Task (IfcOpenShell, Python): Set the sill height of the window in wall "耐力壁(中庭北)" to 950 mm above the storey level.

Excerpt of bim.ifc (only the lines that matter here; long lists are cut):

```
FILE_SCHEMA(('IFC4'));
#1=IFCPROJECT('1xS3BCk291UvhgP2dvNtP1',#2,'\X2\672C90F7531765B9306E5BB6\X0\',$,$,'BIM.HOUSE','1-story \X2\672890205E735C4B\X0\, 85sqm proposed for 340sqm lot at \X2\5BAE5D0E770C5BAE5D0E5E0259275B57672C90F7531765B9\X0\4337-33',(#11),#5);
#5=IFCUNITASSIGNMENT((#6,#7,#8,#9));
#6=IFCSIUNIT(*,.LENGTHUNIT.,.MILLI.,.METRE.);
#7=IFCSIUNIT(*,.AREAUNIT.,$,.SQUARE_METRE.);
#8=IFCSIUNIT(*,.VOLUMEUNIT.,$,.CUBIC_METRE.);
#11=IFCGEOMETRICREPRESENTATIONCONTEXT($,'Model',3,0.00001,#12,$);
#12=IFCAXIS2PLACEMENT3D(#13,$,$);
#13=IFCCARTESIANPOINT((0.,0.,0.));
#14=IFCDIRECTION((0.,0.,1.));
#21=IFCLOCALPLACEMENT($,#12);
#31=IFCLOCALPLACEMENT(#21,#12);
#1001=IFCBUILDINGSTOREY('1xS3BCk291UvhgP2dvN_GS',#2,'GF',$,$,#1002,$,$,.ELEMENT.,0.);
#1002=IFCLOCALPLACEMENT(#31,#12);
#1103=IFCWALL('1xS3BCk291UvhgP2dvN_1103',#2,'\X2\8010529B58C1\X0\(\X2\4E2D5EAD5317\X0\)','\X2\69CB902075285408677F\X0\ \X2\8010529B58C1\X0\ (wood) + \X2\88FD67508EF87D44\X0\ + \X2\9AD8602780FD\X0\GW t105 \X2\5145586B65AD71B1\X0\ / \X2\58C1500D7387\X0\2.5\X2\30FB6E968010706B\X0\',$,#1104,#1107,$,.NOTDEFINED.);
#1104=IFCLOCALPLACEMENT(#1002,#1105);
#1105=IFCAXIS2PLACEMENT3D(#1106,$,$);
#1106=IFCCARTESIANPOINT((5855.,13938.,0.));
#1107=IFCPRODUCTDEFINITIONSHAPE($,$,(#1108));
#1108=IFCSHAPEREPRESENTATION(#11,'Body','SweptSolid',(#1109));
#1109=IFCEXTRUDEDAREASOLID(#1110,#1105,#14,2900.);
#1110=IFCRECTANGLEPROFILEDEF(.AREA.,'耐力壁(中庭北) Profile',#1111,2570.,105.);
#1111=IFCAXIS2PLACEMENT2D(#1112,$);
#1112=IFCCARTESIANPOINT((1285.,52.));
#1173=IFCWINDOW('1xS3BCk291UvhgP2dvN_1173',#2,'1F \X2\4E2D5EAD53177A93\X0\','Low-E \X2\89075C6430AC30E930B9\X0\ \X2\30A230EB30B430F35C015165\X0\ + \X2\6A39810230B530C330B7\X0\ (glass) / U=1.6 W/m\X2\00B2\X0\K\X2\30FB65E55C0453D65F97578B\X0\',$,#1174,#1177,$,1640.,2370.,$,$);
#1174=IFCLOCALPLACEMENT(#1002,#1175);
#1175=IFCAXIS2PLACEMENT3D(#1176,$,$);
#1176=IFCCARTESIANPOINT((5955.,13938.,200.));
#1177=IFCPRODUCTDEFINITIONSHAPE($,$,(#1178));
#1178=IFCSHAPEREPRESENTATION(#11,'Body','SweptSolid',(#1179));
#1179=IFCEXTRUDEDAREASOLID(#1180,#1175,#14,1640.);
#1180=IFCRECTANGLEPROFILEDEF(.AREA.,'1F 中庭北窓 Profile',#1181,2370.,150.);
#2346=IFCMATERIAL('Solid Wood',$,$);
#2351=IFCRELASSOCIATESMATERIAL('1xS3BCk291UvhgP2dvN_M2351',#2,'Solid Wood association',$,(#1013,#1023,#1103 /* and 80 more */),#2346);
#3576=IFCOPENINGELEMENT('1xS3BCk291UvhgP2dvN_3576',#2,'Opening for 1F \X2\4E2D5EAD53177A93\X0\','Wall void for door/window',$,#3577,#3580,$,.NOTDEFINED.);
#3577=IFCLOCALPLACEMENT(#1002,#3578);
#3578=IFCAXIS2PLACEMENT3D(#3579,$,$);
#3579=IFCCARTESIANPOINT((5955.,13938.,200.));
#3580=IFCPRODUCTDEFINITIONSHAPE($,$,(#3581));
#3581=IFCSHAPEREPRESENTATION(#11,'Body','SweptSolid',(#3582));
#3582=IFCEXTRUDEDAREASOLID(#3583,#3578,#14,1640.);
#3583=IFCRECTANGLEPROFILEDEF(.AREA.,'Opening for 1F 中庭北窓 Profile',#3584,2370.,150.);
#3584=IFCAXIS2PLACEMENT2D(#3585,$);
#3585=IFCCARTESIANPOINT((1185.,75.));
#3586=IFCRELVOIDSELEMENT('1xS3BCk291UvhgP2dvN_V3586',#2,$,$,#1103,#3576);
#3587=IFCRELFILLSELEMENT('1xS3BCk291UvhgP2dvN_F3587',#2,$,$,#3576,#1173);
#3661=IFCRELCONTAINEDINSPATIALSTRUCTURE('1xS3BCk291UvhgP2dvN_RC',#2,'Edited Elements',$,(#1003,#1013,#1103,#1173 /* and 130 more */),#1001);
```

```python
import numpy as np
import ifcopenshell
import ifcopenshell.api.geometry
import ifcopenshell.geom
import ifcopenshell.util.element
import ifcopenshell.util.placement
import ifcopenshell.util.shape
import ifcopenshell.util.unit

model = ifcopenshell.open("bim.ifc")
unit_scale = ifcopenshell.util.unit.calculate_unit_scale(model)

window = model.by_id(1173)
opening = window.FillsVoids[0].RelatingOpeningElement
storey = ifcopenshell.util.element.get_container(window, ifc_class="IfcBuildingStorey")
level = ifcopenshell.util.placement.get_local_placement(storey.ObjectPlacement)[2, 3]

# The opening's origin need not be at the sill, so measure its lowest point.
shape = ifcopenshell.geom.create_shape(ifcopenshell.geom.settings(), opening)
bottom = ifcopenshell.util.shape.get_shape_bottom_elevation(shape, shape.geometry) / unit_scale
dz = level + 0.95 / unit_scale - bottom

shift = np.array([0.0, 0.0, dz])
# The window is not placed relative to its opening, so move both.
for product in (opening, window):
    matrix = ifcopenshell.util.placement.get_local_placement(product.ObjectPlacement)
    matrix[:3, 3] += shift
    ifcopenshell.api.geometry.edit_object_placement(model, product=product, matrix=matrix, is_si=False)

print(f"moved by {dz * unit_scale:+.3f} m")

model.write("bim_edited.ifc")
```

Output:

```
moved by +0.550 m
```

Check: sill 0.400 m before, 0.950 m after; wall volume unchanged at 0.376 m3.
